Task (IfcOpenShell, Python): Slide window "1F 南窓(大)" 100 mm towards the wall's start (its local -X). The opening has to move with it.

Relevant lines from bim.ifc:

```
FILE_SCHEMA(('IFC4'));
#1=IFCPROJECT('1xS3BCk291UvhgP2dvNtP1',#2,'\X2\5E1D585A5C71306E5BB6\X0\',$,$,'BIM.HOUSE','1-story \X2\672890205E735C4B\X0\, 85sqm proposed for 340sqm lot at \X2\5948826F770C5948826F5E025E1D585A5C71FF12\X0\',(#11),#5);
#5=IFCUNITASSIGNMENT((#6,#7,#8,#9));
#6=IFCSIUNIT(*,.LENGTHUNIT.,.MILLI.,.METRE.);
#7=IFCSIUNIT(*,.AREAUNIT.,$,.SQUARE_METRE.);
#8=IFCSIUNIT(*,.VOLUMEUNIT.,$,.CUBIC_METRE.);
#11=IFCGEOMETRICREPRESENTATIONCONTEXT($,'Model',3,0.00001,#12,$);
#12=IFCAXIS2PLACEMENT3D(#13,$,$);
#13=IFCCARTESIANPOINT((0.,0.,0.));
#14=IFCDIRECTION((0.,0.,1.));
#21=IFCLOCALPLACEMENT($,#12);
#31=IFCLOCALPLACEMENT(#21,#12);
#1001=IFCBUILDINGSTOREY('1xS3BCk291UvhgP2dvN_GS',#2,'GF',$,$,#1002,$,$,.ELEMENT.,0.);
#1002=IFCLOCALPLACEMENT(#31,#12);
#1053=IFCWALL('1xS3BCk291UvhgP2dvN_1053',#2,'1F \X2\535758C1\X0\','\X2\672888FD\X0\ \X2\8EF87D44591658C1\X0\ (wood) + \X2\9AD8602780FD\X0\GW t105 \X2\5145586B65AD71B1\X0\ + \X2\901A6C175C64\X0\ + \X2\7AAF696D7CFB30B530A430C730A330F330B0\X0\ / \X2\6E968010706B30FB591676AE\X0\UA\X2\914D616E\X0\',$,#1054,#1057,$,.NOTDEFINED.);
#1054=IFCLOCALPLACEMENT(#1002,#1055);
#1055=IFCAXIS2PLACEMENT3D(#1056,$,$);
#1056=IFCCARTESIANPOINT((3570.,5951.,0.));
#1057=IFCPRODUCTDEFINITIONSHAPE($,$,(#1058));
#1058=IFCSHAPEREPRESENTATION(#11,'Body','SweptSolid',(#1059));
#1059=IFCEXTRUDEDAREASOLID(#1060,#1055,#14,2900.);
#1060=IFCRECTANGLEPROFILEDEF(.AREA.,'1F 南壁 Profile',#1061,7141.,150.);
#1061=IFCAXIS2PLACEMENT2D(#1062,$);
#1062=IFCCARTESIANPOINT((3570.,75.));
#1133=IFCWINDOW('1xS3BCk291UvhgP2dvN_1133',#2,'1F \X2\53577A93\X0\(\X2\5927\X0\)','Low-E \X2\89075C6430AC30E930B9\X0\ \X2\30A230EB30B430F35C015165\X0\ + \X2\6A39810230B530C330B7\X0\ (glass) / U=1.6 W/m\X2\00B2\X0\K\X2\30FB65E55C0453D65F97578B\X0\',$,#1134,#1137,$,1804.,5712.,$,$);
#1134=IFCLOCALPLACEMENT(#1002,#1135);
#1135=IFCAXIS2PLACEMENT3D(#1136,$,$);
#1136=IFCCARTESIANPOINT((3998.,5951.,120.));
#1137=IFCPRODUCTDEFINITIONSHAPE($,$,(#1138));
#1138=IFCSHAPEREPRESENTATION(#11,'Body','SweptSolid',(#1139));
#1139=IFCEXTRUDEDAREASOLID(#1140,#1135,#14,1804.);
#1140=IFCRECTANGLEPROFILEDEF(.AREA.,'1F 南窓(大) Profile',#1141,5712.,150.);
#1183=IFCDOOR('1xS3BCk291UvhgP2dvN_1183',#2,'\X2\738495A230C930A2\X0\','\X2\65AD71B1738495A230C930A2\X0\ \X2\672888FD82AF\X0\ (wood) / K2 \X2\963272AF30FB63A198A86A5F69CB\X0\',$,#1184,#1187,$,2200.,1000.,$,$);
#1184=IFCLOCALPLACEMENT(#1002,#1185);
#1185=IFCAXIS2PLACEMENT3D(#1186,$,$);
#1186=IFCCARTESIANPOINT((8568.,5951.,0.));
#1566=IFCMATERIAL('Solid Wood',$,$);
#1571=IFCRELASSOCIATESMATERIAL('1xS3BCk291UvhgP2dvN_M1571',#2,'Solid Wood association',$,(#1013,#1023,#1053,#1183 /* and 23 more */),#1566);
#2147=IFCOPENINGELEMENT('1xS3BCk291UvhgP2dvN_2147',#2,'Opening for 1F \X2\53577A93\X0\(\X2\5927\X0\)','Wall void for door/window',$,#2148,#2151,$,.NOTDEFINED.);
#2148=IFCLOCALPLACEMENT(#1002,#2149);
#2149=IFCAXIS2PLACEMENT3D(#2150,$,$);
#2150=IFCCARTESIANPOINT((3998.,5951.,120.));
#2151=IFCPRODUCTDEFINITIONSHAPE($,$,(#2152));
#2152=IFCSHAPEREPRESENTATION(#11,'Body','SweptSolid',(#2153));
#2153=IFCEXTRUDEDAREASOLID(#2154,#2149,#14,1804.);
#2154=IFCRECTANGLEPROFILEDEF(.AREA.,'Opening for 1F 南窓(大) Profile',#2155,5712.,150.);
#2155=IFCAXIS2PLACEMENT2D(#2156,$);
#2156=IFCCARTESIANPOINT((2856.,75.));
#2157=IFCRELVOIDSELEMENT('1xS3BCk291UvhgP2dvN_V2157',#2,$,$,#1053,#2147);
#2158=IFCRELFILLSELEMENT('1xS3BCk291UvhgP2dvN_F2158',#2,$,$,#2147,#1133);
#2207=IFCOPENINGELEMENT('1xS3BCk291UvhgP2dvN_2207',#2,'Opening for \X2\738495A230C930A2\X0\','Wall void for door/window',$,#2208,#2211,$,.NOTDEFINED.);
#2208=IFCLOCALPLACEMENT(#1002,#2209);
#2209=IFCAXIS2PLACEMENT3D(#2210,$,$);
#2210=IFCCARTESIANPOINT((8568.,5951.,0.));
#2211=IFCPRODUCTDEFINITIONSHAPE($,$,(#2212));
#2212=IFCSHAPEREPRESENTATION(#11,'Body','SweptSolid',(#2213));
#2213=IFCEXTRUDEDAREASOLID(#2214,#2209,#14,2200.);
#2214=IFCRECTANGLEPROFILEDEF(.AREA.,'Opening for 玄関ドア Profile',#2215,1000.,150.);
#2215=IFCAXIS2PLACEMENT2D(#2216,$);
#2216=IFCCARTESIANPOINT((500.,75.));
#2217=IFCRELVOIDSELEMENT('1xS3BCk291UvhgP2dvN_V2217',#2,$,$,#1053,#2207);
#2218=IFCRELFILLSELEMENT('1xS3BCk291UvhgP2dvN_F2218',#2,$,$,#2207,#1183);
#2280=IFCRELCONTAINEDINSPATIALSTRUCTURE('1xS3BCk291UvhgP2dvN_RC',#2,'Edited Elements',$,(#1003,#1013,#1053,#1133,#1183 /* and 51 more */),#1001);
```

```python
import ifcopenshell
import ifcopenshell.api.geometry
import ifcopenshell.util.placement

model = ifcopenshell.open("bim.ifc")

window = model.by_guid("1xS3BCk291UvhgP2dvN_1133")
opening = window.FillsVoids[0].RelatingOpeningElement
wall = opening.VoidsElements[0].RelatingBuildingElement

wall_matrix = ifcopenshell.util.placement.get_local_placement(wall.ObjectPlacement)
shift = wall_matrix[:3, 0] * -100.0
before = ifcopenshell.util.placement.get_local_placement(window.ObjectPlacement)[:3, 3].copy()

# The window is not placed relative to its opening, so move both.
for product in (opening, window):
    matrix = ifcopenshell.util.placement.get_local_placement(product.ObjectPlacement)
    matrix[:3, 3] += shift
    ifcopenshell.api.geometry.edit_object_placement(model, product=product, matrix=matrix, is_si=False)

after = ifcopenshell.util.placement.get_local_placement(window.ObjectPlacement)[:3, 3]
print("window moved by", (after - before).round(3) + 0.0)

model.write("bim_updated.ifc")
```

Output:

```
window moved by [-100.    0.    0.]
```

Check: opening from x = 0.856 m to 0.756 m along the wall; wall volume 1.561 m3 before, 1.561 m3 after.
